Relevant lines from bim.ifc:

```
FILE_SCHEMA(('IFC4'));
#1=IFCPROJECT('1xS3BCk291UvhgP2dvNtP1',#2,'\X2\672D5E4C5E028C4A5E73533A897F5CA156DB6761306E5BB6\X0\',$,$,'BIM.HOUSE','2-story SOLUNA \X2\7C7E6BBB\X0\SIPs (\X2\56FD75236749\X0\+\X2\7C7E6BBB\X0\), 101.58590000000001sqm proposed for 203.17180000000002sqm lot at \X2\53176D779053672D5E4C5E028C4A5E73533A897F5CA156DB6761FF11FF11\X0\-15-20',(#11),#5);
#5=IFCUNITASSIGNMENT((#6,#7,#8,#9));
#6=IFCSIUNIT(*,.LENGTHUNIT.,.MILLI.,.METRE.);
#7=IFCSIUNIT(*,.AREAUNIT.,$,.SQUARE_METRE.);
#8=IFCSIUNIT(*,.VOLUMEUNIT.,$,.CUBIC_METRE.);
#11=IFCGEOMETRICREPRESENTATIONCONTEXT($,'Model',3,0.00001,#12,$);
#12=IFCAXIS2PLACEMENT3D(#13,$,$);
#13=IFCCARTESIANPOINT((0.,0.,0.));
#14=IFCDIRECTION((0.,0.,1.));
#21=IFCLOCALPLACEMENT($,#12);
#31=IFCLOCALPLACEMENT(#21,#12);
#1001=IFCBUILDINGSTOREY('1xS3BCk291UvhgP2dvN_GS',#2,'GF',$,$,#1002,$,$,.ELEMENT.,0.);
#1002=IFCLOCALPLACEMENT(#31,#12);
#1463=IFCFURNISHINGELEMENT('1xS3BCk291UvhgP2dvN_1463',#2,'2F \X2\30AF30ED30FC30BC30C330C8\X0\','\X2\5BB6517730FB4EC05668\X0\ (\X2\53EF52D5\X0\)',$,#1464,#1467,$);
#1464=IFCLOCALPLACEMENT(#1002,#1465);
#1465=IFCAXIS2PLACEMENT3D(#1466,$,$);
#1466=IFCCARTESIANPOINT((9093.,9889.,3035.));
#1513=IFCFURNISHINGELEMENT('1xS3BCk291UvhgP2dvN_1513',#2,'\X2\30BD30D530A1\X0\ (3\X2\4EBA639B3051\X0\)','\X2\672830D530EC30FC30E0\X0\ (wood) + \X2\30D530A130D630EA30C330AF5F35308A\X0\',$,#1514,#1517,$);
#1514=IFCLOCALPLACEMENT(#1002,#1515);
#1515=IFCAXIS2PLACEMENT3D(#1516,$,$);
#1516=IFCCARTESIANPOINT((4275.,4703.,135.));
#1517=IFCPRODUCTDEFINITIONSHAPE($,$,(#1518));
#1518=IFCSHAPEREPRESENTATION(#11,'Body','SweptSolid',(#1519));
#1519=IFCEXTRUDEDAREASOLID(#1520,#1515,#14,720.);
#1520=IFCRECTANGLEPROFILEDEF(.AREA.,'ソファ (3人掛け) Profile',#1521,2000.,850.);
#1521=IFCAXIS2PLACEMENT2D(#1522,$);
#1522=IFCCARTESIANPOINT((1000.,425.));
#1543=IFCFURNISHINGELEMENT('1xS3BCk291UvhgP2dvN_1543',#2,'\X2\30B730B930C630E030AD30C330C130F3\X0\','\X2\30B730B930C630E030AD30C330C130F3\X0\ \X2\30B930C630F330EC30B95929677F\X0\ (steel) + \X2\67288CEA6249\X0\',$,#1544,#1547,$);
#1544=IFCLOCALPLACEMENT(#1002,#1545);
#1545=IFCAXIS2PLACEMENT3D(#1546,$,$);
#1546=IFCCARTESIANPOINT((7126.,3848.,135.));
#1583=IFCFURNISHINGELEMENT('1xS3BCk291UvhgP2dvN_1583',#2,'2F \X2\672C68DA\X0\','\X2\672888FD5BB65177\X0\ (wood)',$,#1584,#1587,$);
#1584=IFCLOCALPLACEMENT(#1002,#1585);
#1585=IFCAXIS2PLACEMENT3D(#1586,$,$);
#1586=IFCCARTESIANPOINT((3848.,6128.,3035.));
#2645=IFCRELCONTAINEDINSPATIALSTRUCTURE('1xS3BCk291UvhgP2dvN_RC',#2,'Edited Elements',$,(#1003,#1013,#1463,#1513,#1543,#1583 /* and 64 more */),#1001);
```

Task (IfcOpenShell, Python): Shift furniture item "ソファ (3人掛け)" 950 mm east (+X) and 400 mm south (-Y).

```python
import ifcopenshell
import ifcopenshell.api.geometry
import ifcopenshell.util.placement
import ifcopenshell.util.unit

model = ifcopenshell.open("bim.ifc")
unit_scale = ifcopenshell.util.unit.calculate_unit_scale(model)

item = model.by_id(1513)
matrix = ifcopenshell.util.placement.get_local_placement(item.ObjectPlacement)
matrix[0, 3] += 0.95 / unit_scale
matrix[1, 3] -= 0.4 / unit_scale
ifcopenshell.api.geometry.edit_object_placement(model, product=item, matrix=matrix, is_si=False)

print(ifcopenshell.util.placement.get_local_placement(item.ObjectPlacement).round(3) + 0.0)

model.write("bim_rev.ifc")
```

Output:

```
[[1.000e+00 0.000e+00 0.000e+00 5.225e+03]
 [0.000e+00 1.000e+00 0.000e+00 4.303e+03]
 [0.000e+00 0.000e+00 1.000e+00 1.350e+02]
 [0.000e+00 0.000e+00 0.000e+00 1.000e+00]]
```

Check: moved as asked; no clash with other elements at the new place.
